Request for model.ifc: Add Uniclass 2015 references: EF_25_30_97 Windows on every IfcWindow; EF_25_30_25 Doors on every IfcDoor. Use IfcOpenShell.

First a look at what the model holds.

```python
import ifcopenshell

model = ifcopenshell.open("model.ifc")
print(model.schema)
print("classifications:", [c.Name for c in model.by_type("IfcClassification")])
for ifc_class in ("IfcDoor", "IfcRoof", "IfcStair", "IfcWall", "IfcWindow"):
    print(ifc_class, len(model.by_type(ifc_class)))
```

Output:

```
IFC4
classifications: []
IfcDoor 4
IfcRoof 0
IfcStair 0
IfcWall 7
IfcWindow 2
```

```python
import ifcopenshell
import ifcopenshell.api.classification

model = ifcopenshell.open("model.ifc")

system = ifcopenshell.api.classification.add_classification(model, classification="Uniclass 2015")

codes = {
    "IfcWindow": ("EF_25_30_97", "Windows"),
    "IfcDoor": ("EF_25_30_25", "Doors"),
}
for ifc_class, (code, name) in codes.items():
    products = model.by_type(ifc_class)
    ifcopenshell.api.classification.add_reference(
        model, products=products, classification=system, identification=code, name=name
    )
    print(code, len(products))

model.write("model_v2.ifc")
```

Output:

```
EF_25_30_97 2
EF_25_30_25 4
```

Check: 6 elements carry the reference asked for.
